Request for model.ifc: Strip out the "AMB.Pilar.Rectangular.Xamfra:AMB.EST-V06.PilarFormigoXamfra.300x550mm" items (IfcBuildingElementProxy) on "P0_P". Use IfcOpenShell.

First a look at what the model holds.

```python
import ifcopenshell
import ifcopenshell.util.element

model = ifcopenshell.open("model.ifc")
print(model.schema)
storey = next(s for s in model.by_type("IfcBuildingStorey") if s.Name == "P0_P")
proxies = [e for e in ifcopenshell.util.element.get_decomposition(storey) if e.is_a("IfcBuildingElementProxy")]
seen = {}
for e in proxies:
    element_type = ifcopenshell.util.element.get_type(e)
    name = element_type.Name if element_type not in (None, e) else None
    seen[name] = seen.get(name, 0) + 1
for name, count in sorted(seen.items(), key=str):
    print(count, "x", name)
```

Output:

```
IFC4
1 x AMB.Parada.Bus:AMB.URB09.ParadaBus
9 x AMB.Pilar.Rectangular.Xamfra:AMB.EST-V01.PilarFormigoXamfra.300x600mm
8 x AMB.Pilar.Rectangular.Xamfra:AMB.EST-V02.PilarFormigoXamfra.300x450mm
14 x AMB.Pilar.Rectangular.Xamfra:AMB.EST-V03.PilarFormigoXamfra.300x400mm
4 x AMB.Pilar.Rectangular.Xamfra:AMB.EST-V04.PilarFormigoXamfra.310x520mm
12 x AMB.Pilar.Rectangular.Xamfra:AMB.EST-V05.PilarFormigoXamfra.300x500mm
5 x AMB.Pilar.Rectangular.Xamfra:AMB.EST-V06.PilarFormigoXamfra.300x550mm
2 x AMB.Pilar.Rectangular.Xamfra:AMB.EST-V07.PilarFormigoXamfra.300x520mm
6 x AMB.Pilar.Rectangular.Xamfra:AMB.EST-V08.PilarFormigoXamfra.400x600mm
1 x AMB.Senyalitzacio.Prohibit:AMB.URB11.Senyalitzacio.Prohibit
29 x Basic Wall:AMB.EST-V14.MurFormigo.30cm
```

```python
import ifcopenshell
import ifcopenshell.api.root
import ifcopenshell.util.element

model = ifcopenshell.open("model.ifc")

storey = next(s for s in model.by_type("IfcBuildingStorey") if s.Name == "P0_P")
proxies = [e for e in ifcopenshell.util.element.get_decomposition(storey) if e.is_a("IfcBuildingElementProxy")]
targets = [e for e in proxies if (t := ifcopenshell.util.element.get_type(e)) not in (None, e) and t.Name == "AMB.Pilar.Rectangular.Xamfra:AMB.EST-V06.PilarFormigoXamfra.300x550mm"]

for e in targets:
    ifcopenshell.api.root.remove_product(model, product=e)
print(len(targets), "removed")

model.write("model_rev.ifc")
```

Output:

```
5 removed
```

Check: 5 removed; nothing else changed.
